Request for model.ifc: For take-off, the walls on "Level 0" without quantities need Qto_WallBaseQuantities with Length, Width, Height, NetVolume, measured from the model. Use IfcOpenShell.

First a look at what the model holds.

```python
import ifcopenshell
import ifcopenshell.util.element
import ifcopenshell.util.unit

model = ifcopenshell.open("model.ifc")
print(model.schema)
for unit_type in ("LENGTHUNIT", "AREAUNIT", "VOLUMEUNIT"):
    print(unit_type, ifcopenshell.util.unit.calculate_unit_scale(model, unit_type))
storey = next(s for s in model.by_type("IfcBuildingStorey") if s.Name == "Level 0")
walls = [e for e in ifcopenshell.util.element.get_decomposition(storey) if e.is_a("IfcWall")]
for e in sorted(walls, key=lambda e: e.id()):
    print(e.id(), e.is_a(), e.Name, list(ifcopenshell.util.element.get_psets(e, qtos_only=True)), sep=" | ")
```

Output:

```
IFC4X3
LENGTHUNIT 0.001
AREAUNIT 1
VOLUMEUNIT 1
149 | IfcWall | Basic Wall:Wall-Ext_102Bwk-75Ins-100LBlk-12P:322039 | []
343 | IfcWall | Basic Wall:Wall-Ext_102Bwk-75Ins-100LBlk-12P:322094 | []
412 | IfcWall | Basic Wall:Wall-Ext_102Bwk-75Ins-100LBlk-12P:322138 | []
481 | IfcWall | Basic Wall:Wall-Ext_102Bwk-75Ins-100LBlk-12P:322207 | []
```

```python
import ifcopenshell
import ifcopenshell.api.pset
import ifcopenshell.geom
import ifcopenshell.util.element
import ifcopenshell.util.shape
import ifcopenshell.util.unit

model = ifcopenshell.open("model.ifc")
unit_scale = ifcopenshell.util.unit.calculate_unit_scale(model)
volume_scale = ifcopenshell.util.unit.calculate_unit_scale(model, "VOLUMEUNIT")
settings = ifcopenshell.geom.settings()

storey = next(s for s in model.by_type("IfcBuildingStorey") if s.Name == "Level 0")
walls = [e for e in ifcopenshell.util.element.get_decomposition(storey) if e.is_a("IfcWall")]

for e in sorted(walls, key=lambda e: e.id()):
    if ifcopenshell.util.element.get_psets(e, qtos_only=True, should_inherit=False):
        continue
    # Geometry comes back in metres, in the element's own axes.
    shape = ifcopenshell.geom.create_shape(settings, e)
    values = {
        "Length": ifcopenshell.util.shape.get_x(shape.geometry) / unit_scale,
        "Width": ifcopenshell.util.shape.get_y(shape.geometry) / unit_scale,
        "Height": ifcopenshell.util.shape.get_z(shape.geometry) / unit_scale,
        "NetVolume": ifcopenshell.util.shape.get_volume(shape.geometry) / volume_scale,
    }
    qto = ifcopenshell.api.pset.add_qto(model, product=e, name="Qto_WallBaseQuantities")
    ifcopenshell.api.pset.edit_qto(model, qto=qto, properties=values)
    print(e.id(), {k: round(v, 3) for k, v in values.items()})

model.write("model_updated.ifc")
```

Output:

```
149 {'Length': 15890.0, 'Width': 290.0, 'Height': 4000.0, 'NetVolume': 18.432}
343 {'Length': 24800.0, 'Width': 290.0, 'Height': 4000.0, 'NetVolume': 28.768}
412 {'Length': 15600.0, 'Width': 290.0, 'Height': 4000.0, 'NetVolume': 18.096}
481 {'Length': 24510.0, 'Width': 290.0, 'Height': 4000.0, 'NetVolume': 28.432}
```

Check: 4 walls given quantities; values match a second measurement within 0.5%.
